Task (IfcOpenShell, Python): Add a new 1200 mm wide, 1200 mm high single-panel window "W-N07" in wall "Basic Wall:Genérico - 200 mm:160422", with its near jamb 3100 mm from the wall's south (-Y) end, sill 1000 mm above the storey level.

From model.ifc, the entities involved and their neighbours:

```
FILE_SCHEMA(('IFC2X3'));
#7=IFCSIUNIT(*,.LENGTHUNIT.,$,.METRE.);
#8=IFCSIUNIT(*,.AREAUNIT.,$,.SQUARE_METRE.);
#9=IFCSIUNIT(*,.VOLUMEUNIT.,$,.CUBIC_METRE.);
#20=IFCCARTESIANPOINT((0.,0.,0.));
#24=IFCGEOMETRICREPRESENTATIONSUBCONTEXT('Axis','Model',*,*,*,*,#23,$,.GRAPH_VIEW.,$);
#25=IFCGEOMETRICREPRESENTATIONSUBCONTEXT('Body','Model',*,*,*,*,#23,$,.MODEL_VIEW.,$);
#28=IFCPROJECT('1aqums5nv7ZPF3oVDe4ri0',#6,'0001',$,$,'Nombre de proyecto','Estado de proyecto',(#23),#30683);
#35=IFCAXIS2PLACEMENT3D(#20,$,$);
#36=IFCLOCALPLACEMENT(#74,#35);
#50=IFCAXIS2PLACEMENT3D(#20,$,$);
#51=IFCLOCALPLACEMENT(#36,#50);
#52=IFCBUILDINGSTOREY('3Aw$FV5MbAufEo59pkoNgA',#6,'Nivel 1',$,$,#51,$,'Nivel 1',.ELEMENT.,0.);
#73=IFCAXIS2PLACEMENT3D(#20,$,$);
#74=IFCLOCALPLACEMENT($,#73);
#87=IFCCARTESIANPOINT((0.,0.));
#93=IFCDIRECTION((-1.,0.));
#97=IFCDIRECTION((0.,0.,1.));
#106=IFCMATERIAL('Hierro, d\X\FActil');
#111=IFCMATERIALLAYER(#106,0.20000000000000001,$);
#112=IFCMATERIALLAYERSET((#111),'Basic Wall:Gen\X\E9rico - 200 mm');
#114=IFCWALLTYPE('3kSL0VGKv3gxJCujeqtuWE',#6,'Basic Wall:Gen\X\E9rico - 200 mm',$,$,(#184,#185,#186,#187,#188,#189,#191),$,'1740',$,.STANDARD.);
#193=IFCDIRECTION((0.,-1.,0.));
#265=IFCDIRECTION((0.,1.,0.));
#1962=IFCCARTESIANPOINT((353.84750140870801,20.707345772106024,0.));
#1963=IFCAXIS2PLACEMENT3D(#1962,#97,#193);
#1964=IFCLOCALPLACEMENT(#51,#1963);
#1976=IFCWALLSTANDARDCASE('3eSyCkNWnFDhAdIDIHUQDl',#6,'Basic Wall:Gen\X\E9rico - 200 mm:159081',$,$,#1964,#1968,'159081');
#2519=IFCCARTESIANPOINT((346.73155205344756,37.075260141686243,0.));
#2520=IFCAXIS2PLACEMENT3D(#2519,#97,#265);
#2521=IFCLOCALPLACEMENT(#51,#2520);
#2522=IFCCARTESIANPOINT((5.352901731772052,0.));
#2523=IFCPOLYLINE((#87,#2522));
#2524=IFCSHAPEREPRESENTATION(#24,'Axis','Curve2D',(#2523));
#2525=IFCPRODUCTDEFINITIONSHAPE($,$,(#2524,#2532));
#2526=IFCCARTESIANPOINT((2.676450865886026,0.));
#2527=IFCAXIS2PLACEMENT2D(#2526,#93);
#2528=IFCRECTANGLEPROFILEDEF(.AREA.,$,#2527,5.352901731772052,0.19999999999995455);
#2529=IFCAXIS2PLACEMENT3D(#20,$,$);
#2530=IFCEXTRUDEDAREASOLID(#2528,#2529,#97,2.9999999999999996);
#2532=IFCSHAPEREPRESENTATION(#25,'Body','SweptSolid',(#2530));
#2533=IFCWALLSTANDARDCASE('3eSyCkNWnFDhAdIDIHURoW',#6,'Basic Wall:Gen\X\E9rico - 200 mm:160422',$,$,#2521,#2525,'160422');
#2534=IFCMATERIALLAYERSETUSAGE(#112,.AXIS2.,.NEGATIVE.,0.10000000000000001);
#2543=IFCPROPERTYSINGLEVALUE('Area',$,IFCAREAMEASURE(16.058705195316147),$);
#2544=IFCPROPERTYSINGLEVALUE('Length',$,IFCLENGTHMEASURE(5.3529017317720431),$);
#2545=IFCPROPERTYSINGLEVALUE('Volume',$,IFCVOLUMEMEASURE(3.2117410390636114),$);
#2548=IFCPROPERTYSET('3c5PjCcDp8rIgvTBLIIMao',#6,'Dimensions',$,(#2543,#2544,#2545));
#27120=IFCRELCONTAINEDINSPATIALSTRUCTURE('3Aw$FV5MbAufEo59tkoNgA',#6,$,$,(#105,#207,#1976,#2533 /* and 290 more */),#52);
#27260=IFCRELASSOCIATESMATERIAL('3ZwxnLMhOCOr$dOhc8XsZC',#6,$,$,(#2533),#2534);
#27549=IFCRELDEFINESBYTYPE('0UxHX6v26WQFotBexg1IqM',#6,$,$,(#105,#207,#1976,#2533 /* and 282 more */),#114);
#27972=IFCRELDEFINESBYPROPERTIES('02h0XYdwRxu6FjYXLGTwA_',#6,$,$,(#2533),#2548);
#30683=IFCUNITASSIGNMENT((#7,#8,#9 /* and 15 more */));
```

```python
import numpy as np
import ifcopenshell
import ifcopenshell.api.feature
import ifcopenshell.api.geometry
import ifcopenshell.api.pset
import ifcopenshell.api.root
import ifcopenshell.api.spatial
import ifcopenshell.api.type
import ifcopenshell.geom
import ifcopenshell.util.element
import ifcopenshell.util.placement
import ifcopenshell.util.representation
import ifcopenshell.util.shape
import ifcopenshell.util.unit

model = ifcopenshell.open("model.ifc")
unit_scale = ifcopenshell.util.unit.calculate_unit_scale(model)
area_scale = ifcopenshell.util.unit.calculate_unit_scale(model, "AREAUNIT")
volume_scale = ifcopenshell.util.unit.calculate_unit_scale(model, "VOLUMEUNIT")
settings = ifcopenshell.geom.settings()


def volume(element):
    """Net volume in cubic metres, openings subtracted."""
    shape = ifcopenshell.geom.create_shape(settings, element)
    return ifcopenshell.util.shape.get_volume(shape.geometry)


wall = model.by_guid("3eSyCkNWnFDhAdIDIHURoW")
storey = ifcopenshell.util.element.get_container(wall, ifc_class="IfcBuildingStorey")
context = ifcopenshell.util.representation.get_context(model, "Model", "Body", "MODEL_VIEW")
before = volume(wall)

width, height, from_end, sill = 1.2, 1.2, 3.1, 1  # metres

# The wall runs along its own X axis, and the end named is its -X end.
wall_shape = ifcopenshell.geom.create_shape(settings, wall)
x, y, z = ifcopenshell.util.shape.get_vertices(wall_shape.geometry).T
start = x.min() + from_end
face, thickness = float(y.min()), float(y.max() - y.min())
wall_matrix = ifcopenshell.util.placement.get_local_placement(wall.ObjectPlacement)
level = ifcopenshell.util.placement.get_local_placement(storey.ObjectPlacement)[2, 3]


def in_wall(x, y):
    """Placement at x, y metres in the wall's axes, at sill height."""
    matrix = wall_matrix.copy()
    matrix[:, 3] = wall_matrix @ np.array([x / unit_scale, y / unit_scale, 0.0, 1.0])
    matrix[2, 3] = level + sill / unit_scale
    return matrix


# Opening: a box that overshoots both wall faces by 50 mm.
opening = ifcopenshell.api.root.create_entity(model, ifc_class="IfcOpeningElement")
box = ifcopenshell.api.geometry.add_wall_representation(
    model, context=context, length=width, height=height, thickness=thickness + 0.1
)
ifcopenshell.api.geometry.assign_representation(model, product=opening, representation=box)
ifcopenshell.api.geometry.edit_object_placement(model, product=opening, matrix=in_wall(start, face - 0.05), is_si=False)
ifcopenshell.api.feature.add_feature(model, feature=opening, element=wall)

window = ifcopenshell.api.root.create_entity(model, ifc_class="IfcWindow", name="W-N07")
window.OverallWidth, window.OverallHeight = width / unit_scale, height / unit_scale
body = ifcopenshell.api.geometry.add_window_representation(
    model,
    context=context,
    overall_width=window.OverallWidth,
    overall_height=window.OverallHeight,
    partition_type="SINGLE_PANEL",
)
ifcopenshell.api.geometry.assign_representation(model, product=window, representation=body)
ifcopenshell.api.spatial.assign_container(model, products=[window], relating_structure=storey)
fills = ifcopenshell.api.feature.add_filling(model, opening=opening, element=window)
fills.OwnerHistory = window.OwnerHistory  # required in IFC2X3

# IFC2X3 keeps the operation on the window style.
style = ifcopenshell.api.root.create_entity(model, ifc_class="IfcWindowStyle", name="W-N07")
style.OperationType, style.ConstructionType = "SINGLE_PANEL", "NOTDEFINED"
style.ParameterTakesPrecedence = style.Sizeable = False
ifcopenshell.api.type.assign_type(model, related_objects=[window], relating_type=style)

# Centre the window in the wall's thickness.
ifcopenshell.api.geometry.edit_object_placement(model, product=window, matrix=in_wall(start, face), is_si=False)
window_shape = ifcopenshell.geom.create_shape(settings, window)
depth = ifcopenshell.util.shape.get_vertices(window_shape.geometry)[:, 1]
offset = face + thickness / 2 - (depth.min() + depth.max()) / 2
ifcopenshell.api.geometry.edit_object_placement(model, product=window, matrix=in_wall(start, offset), is_si=False)

after = volume(wall)

# Update the wall's stored quantities.
pset = model.by_id(ifcopenshell.util.element.get_pset(wall, "Dimensions", should_inherit=False)["id"])
ifcopenshell.api.pset.edit_pset(model, pset=pset, properties={
    "Area": model.create_entity("IfcAreaMeasure", after / thickness / area_scale),
    "Volume": model.create_entity("IfcVolumeMeasure", after / volume_scale),
})

print(f"wall volume {before:.3f} -> {after:.3f} m3")

model.write("model_edited.ifc")
```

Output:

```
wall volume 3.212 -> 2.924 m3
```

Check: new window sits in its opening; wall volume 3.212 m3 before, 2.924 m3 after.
